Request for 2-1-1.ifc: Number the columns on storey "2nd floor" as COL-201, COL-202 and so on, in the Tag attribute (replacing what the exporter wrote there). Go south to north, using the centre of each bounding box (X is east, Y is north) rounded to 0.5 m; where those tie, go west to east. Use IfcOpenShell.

First a look at what the model holds.

```python
import ifcopenshell
import ifcopenshell.util.element
import ifcopenshell.util.placement

model = ifcopenshell.open("2-1-1.ifc")
print(model.schema)
storey = next(s for s in model.by_type("IfcBuildingStorey") if s.Name == "2nd floor")
columns = [e for e in ifcopenshell.util.element.get_decomposition(storey) if e.is_a("IfcColumn")]
for e in sorted(columns, key=lambda e: e.id()):
    origin = ifcopenshell.util.placement.get_local_placement(e.ObjectPlacement)[:3, 3]
    print(e.id(), e.Tag, e.Name, origin.round(2) + 0.0, sep=" | ")
```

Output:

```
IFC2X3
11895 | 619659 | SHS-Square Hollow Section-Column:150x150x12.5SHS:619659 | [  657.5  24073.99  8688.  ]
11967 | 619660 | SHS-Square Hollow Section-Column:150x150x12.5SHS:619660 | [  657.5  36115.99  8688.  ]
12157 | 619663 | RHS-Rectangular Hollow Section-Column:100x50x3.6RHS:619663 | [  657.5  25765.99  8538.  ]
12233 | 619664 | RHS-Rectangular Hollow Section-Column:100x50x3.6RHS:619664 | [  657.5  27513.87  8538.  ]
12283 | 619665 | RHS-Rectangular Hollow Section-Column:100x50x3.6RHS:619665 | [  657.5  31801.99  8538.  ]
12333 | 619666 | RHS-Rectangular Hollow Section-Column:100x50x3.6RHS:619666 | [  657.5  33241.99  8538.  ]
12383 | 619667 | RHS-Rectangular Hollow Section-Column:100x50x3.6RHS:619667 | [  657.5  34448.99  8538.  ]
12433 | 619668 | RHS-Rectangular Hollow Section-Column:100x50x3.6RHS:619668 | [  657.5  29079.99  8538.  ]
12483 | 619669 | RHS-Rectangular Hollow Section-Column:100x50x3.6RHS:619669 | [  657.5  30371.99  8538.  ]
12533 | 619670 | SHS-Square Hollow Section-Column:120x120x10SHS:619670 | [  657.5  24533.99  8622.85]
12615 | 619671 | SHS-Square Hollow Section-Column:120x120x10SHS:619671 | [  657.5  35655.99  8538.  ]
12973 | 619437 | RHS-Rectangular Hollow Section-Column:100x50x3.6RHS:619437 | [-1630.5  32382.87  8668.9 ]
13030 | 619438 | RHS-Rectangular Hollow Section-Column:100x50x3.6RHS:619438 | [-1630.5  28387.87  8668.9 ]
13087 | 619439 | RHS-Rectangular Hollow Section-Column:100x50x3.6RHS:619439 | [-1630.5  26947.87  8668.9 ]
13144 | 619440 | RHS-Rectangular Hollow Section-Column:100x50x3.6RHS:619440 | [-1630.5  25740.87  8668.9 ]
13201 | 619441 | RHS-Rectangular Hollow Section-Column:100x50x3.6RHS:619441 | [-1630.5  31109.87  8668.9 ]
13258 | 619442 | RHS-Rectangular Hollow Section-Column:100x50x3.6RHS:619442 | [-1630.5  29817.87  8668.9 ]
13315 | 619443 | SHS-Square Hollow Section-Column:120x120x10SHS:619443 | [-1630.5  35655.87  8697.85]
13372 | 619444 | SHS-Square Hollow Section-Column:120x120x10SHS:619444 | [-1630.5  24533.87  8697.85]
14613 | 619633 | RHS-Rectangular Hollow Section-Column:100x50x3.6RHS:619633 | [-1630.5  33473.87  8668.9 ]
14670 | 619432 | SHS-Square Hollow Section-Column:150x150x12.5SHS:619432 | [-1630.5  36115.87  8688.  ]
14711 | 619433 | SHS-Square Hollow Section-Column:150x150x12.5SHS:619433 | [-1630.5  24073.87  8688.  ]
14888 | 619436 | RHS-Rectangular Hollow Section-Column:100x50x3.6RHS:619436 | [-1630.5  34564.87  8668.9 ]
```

```python
import ifcopenshell
import ifcopenshell.geom
import ifcopenshell.util.element
import ifcopenshell.util.shape

model = ifcopenshell.open("2-1-1.ifc")
settings = ifcopenshell.geom.settings()
settings.set("use-world-coords", True)


def centre(element):
    shape = ifcopenshell.geom.create_shape(settings, element)
    return ifcopenshell.util.shape.get_bbox_centroid(shape.geometry)


storey = next(s for s in model.by_type("IfcBuildingStorey") if s.Name == "2nd floor")
columns = [e for e in ifcopenshell.util.element.get_decomposition(storey) if e.is_a("IfcColumn")]

# Insertion points can sit at a corner or the storey origin, so sort by the geometry (in metres).
centres = {e: centre(e) for e in columns}
columns.sort(key=lambda e: (round(centres[e][1] / 0.5), centres[e][0]))

for i, e in enumerate(columns, start=1):
    number = f"COL-2{i:02d}"
    e.Tag = number
    print(e.id(), number)

model.write("2-1-1-out.ifc")
```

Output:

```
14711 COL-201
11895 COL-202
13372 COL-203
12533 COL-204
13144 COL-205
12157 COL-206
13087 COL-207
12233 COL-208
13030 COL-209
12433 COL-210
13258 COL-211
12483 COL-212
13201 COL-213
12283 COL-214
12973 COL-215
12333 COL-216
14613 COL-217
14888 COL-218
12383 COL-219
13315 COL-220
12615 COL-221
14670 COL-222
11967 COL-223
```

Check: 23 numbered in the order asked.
